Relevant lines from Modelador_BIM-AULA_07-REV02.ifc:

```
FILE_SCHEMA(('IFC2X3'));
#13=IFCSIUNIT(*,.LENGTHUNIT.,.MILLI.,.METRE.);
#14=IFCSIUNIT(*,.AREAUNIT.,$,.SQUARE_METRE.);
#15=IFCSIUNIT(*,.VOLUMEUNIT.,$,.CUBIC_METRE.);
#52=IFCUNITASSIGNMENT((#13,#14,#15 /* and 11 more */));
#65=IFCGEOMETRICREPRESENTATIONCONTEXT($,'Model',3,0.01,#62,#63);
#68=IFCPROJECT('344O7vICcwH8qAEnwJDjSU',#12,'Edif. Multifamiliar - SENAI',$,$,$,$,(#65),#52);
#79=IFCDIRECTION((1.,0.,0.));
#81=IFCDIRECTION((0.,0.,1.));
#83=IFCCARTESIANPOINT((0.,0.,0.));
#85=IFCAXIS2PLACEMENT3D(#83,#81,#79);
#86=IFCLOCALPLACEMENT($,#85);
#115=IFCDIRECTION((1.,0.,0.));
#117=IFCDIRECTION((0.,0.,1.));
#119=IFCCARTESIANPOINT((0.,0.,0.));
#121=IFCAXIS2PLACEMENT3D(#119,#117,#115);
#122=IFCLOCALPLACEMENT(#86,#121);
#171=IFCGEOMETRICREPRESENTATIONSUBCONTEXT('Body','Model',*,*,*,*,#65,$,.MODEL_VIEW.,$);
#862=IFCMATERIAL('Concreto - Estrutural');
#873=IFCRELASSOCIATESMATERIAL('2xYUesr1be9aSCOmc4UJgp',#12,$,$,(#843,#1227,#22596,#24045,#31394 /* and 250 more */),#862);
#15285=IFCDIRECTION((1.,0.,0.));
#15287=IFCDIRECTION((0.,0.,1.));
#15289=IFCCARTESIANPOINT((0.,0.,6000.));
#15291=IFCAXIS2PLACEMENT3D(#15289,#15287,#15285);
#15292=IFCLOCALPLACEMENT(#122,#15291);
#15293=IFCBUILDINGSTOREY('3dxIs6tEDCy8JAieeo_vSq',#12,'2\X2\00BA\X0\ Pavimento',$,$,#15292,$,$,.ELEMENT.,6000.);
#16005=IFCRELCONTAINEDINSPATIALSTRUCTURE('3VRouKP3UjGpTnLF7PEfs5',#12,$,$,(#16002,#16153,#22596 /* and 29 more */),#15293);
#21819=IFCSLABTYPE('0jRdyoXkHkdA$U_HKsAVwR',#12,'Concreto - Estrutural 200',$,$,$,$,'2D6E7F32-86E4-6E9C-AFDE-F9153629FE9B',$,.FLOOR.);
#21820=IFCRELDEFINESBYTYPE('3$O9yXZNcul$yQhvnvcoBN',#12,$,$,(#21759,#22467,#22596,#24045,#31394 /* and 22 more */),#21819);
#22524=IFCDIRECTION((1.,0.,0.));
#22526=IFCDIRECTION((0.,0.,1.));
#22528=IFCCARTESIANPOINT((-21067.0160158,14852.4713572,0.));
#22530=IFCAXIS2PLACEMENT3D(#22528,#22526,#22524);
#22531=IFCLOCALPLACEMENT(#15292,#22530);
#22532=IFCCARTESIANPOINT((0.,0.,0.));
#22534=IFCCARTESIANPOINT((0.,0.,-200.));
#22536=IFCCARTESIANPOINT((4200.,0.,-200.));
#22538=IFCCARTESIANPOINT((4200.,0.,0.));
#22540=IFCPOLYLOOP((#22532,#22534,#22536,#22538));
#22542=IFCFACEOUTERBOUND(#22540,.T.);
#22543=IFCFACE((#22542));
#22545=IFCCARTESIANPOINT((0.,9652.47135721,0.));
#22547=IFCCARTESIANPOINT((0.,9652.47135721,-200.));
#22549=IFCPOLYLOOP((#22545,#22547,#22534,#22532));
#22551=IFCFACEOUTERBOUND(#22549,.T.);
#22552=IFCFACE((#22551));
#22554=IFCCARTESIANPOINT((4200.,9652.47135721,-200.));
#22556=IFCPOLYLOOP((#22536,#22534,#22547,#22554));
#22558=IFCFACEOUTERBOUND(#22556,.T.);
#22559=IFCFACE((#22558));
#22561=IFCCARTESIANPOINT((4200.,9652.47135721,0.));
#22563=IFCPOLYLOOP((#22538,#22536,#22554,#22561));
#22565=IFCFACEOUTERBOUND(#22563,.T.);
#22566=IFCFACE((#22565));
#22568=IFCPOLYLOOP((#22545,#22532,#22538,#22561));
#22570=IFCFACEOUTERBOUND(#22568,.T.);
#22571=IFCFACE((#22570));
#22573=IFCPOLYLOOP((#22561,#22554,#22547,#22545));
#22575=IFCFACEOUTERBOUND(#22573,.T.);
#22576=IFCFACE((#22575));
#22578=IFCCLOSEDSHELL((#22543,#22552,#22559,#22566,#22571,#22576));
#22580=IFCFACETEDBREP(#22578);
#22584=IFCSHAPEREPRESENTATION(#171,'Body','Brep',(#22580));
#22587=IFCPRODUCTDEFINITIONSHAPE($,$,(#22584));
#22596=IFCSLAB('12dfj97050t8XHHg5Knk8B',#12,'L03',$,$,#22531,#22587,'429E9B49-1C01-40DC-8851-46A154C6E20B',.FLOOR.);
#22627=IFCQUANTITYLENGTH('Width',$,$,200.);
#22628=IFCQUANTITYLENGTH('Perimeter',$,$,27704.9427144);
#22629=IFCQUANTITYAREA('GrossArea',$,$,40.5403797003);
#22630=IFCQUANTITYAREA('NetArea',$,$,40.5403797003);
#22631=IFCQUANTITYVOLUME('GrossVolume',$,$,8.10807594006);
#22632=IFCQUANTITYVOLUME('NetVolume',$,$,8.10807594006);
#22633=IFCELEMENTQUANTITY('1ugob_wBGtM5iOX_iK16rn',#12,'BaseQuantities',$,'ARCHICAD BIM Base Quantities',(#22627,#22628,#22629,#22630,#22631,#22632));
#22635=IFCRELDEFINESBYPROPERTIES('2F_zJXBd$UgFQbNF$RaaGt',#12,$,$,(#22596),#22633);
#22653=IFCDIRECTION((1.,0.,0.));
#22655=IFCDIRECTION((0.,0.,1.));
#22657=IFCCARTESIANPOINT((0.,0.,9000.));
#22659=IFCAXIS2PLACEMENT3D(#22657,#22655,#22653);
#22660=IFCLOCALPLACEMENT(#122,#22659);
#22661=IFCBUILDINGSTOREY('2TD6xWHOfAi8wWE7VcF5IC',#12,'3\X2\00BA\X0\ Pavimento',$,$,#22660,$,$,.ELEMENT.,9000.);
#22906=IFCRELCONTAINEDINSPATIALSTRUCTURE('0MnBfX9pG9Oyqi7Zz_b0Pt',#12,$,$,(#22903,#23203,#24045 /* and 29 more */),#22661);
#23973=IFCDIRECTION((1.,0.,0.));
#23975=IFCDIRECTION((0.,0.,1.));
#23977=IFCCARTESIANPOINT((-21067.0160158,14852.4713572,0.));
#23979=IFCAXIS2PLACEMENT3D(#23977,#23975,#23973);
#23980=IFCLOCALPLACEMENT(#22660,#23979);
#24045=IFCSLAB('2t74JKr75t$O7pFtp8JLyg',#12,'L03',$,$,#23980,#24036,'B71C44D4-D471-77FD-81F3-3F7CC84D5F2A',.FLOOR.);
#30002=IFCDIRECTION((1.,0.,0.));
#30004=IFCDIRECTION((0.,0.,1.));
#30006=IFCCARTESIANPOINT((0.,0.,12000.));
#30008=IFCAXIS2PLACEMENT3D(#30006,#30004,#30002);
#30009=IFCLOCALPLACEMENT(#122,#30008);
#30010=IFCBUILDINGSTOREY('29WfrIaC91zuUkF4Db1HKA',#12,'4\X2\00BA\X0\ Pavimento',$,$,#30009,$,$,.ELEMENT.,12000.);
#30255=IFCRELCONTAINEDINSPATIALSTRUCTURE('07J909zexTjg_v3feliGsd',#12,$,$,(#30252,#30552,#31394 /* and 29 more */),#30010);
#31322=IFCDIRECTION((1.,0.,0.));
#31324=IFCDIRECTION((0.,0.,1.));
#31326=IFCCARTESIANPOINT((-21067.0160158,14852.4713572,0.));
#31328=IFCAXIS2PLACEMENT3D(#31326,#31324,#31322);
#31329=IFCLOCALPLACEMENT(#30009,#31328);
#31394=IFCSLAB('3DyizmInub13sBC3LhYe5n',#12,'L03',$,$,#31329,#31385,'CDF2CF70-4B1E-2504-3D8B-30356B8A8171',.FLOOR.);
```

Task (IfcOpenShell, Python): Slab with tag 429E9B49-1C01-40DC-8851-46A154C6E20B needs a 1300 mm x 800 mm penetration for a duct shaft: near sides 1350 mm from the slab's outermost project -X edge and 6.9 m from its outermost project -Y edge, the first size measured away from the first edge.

```python
import numpy as np
import ifcopenshell
import ifcopenshell.api.feature
import ifcopenshell.api.geometry
import ifcopenshell.api.pset
import ifcopenshell.api.root
import ifcopenshell.geom
import ifcopenshell.util.element
import ifcopenshell.util.placement
import ifcopenshell.util.representation
import ifcopenshell.util.shape
import ifcopenshell.util.unit

model = ifcopenshell.open("Modelador_BIM-AULA_07-REV02.ifc")
unit_scale = ifcopenshell.util.unit.calculate_unit_scale(model)
area_scale = ifcopenshell.util.unit.calculate_unit_scale(model, "AREAUNIT")
volume_scale = ifcopenshell.util.unit.calculate_unit_scale(model, "VOLUMEUNIT")
settings = ifcopenshell.geom.settings()


def volume(element):
    """Net volume in cubic metres, openings subtracted."""
    shape = ifcopenshell.geom.create_shape(settings, element)
    return ifcopenshell.util.shape.get_volume(shape.geometry)


slab = model.by_guid("12dfj97050t8XHHg5Knk8B")
before = volume(slab)

# Extent in the slab's own axes, in metres. The edges named are its -X and -Y sides.
slab_shape = ifcopenshell.geom.create_shape(settings, slab)
vertices = ifcopenshell.util.shape.get_vertices(slab_shape.geometry)
x_min, y_min, bottom = vertices.min(axis=0)
top = vertices[:, 2].max()

opening = ifcopenshell.api.root.create_entity(model, ifc_class="IfcOpeningElement", name="Duct shaft opening")
context = ifcopenshell.util.representation.get_context(model, "Model", "Body", "MODEL_VIEW")
width, depth = 1.3, 0.8
outline = [(0.0, 0.0), (width, 0.0), (width, depth), (0.0, depth), (0.0, 0.0)]
# Overshoot both faces by 50 mm so the cut is clean.
shape = ifcopenshell.api.geometry.add_slab_representation(
    model, context=context, depth=top - bottom + 0.1, polyline=outline
)
ifcopenshell.api.geometry.assign_representation(model, product=opening, representation=shape)

matrix = ifcopenshell.util.placement.get_local_placement(slab.ObjectPlacement)
matrix[:, 3] = matrix @ np.append(np.array([x_min + 1.35, y_min + 6.9, bottom - 0.05]) / unit_scale, 1.0)
ifcopenshell.api.geometry.edit_object_placement(model, product=opening, matrix=matrix, is_si=False)
ifcopenshell.api.feature.add_feature(model, feature=opening, element=slab)

after = volume(slab)

# Update the slab's stored quantities.
qto = model.by_id(ifcopenshell.util.element.get_pset(slab, "BaseQuantities", should_inherit=False)["id"])
ifcopenshell.api.pset.edit_qto(model, qto=qto, properties={
    "NetArea": after / (top - bottom) / area_scale,
    "NetVolume": after / volume_scale,
})

print(f"slab volume {before:.3f} -> {after:.3f} m3")

model.write("Modelador_BIM-AULA_07-REV02_edited.ifc")
```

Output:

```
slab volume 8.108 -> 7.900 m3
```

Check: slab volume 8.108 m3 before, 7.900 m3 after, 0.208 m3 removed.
